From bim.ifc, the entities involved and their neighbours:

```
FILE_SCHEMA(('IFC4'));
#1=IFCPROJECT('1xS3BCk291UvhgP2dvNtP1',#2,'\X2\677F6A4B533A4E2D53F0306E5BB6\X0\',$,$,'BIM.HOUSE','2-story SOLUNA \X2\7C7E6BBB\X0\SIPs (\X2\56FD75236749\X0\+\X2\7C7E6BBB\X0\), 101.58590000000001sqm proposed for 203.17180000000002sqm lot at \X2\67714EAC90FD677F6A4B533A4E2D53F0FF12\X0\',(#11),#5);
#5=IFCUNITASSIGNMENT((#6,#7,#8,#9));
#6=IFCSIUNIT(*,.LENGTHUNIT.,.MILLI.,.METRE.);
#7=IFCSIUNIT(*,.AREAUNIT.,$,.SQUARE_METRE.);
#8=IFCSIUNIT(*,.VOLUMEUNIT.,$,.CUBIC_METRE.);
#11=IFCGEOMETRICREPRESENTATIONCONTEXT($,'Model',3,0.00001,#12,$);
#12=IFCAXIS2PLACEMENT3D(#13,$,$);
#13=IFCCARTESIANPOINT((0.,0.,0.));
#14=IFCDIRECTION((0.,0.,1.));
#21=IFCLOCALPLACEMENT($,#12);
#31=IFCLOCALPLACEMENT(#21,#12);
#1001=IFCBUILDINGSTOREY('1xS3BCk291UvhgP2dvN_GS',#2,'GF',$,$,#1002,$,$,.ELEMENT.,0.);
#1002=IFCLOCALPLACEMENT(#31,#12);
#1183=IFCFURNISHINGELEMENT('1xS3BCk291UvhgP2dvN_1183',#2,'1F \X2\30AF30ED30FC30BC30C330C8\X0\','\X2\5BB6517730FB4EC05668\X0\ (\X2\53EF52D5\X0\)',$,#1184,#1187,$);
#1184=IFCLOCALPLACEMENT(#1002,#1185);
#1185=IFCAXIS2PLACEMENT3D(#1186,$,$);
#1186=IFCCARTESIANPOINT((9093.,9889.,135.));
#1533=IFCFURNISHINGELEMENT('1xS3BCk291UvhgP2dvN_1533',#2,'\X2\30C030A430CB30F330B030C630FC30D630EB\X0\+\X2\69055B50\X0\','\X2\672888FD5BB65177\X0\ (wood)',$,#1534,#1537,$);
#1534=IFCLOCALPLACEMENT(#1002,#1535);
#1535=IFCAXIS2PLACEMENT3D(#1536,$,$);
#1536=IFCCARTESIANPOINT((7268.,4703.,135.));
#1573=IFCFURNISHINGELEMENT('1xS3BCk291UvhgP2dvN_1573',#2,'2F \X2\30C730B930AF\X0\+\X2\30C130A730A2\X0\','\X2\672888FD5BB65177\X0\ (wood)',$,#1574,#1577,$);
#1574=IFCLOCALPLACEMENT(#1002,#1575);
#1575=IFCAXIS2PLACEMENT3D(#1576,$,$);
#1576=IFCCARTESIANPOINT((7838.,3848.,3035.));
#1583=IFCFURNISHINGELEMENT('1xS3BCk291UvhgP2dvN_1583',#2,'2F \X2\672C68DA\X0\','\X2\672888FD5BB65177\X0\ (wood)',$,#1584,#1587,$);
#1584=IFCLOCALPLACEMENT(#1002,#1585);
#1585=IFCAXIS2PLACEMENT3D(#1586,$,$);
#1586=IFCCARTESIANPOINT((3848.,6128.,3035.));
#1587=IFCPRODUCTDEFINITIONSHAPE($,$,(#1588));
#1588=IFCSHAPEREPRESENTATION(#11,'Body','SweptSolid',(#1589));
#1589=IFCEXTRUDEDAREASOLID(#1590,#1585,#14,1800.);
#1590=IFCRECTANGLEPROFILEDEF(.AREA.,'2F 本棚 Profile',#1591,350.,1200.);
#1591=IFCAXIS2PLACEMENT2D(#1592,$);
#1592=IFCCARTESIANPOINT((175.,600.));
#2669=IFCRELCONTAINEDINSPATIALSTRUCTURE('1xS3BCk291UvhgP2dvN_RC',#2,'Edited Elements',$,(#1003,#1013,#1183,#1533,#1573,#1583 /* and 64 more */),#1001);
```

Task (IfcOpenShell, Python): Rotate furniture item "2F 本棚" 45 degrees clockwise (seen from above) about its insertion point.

```python
import ifcopenshell
import ifcopenshell.api.geometry
import ifcopenshell.util.placement

model = ifcopenshell.open("bim.ifc")

item = model.by_guid("1xS3BCk291UvhgP2dvN_1583")
matrix = ifcopenshell.util.placement.get_local_placement(item.ObjectPlacement)
matrix = matrix @ ifcopenshell.util.placement.rotation(-45, "Z")
ifcopenshell.api.geometry.edit_object_placement(model, product=item, matrix=matrix, is_si=False)

print(ifcopenshell.util.placement.get_local_placement(item.ObjectPlacement).round(3) + 0.0)

model.write("bim_rev.ifc")
```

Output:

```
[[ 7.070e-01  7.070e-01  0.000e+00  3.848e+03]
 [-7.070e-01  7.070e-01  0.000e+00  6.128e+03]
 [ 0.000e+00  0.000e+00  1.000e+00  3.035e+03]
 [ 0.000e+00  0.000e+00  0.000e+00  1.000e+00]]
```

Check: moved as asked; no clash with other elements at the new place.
